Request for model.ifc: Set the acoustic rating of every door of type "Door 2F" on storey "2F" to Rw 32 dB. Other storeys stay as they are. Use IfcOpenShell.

First a look at what the model holds.

```python
import ifcopenshell
import ifcopenshell.util.element

model = ifcopenshell.open("model.ifc")
print(model.schema)
storey = next(s for s in model.by_type("IfcBuildingStorey") if s.Name == "2F")
doors = [e for e in ifcopenshell.util.element.get_decomposition(storey) if e.is_a("IfcDoor")]
seen = {}
for e in doors:
    element_type = ifcopenshell.util.element.get_type(e)
    key = (element_type.Name if element_type != e and element_type else None, ifcopenshell.util.element.get_pset(e, "Pset_DoorCommon", "AcousticRating"))
    seen[key] = seen.get(key, 0) + 1
for (name, value), count in sorted(seen.items(), key=str):
    print(count, "x", name, "|", value)
```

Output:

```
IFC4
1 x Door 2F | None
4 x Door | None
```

```python
import ifcopenshell
import ifcopenshell.api.pset
import ifcopenshell.util.element

model = ifcopenshell.open("model.ifc")

storey = next(s for s in model.by_type("IfcBuildingStorey") if s.Name == "2F")
doors = [e for e in ifcopenshell.util.element.get_decomposition(storey) if e.is_a("IfcDoor")]

count = 0
for e in doors:
    element_type = ifcopenshell.util.element.get_type(e)
    if element_type in (None, e) or element_type.Name != "Door 2F":
        continue
    # add_pset returns the element's existing set when there is one.
    pset = ifcopenshell.api.pset.add_pset(model, product=e, name="Pset_DoorCommon")
    ifcopenshell.api.pset.edit_pset(model, pset=pset, properties={"AcousticRating": "Rw 32 dB"})
    count += 1

print(count, "doors updated")

model.write("model-out.ifc")
```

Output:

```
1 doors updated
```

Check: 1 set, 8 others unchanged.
